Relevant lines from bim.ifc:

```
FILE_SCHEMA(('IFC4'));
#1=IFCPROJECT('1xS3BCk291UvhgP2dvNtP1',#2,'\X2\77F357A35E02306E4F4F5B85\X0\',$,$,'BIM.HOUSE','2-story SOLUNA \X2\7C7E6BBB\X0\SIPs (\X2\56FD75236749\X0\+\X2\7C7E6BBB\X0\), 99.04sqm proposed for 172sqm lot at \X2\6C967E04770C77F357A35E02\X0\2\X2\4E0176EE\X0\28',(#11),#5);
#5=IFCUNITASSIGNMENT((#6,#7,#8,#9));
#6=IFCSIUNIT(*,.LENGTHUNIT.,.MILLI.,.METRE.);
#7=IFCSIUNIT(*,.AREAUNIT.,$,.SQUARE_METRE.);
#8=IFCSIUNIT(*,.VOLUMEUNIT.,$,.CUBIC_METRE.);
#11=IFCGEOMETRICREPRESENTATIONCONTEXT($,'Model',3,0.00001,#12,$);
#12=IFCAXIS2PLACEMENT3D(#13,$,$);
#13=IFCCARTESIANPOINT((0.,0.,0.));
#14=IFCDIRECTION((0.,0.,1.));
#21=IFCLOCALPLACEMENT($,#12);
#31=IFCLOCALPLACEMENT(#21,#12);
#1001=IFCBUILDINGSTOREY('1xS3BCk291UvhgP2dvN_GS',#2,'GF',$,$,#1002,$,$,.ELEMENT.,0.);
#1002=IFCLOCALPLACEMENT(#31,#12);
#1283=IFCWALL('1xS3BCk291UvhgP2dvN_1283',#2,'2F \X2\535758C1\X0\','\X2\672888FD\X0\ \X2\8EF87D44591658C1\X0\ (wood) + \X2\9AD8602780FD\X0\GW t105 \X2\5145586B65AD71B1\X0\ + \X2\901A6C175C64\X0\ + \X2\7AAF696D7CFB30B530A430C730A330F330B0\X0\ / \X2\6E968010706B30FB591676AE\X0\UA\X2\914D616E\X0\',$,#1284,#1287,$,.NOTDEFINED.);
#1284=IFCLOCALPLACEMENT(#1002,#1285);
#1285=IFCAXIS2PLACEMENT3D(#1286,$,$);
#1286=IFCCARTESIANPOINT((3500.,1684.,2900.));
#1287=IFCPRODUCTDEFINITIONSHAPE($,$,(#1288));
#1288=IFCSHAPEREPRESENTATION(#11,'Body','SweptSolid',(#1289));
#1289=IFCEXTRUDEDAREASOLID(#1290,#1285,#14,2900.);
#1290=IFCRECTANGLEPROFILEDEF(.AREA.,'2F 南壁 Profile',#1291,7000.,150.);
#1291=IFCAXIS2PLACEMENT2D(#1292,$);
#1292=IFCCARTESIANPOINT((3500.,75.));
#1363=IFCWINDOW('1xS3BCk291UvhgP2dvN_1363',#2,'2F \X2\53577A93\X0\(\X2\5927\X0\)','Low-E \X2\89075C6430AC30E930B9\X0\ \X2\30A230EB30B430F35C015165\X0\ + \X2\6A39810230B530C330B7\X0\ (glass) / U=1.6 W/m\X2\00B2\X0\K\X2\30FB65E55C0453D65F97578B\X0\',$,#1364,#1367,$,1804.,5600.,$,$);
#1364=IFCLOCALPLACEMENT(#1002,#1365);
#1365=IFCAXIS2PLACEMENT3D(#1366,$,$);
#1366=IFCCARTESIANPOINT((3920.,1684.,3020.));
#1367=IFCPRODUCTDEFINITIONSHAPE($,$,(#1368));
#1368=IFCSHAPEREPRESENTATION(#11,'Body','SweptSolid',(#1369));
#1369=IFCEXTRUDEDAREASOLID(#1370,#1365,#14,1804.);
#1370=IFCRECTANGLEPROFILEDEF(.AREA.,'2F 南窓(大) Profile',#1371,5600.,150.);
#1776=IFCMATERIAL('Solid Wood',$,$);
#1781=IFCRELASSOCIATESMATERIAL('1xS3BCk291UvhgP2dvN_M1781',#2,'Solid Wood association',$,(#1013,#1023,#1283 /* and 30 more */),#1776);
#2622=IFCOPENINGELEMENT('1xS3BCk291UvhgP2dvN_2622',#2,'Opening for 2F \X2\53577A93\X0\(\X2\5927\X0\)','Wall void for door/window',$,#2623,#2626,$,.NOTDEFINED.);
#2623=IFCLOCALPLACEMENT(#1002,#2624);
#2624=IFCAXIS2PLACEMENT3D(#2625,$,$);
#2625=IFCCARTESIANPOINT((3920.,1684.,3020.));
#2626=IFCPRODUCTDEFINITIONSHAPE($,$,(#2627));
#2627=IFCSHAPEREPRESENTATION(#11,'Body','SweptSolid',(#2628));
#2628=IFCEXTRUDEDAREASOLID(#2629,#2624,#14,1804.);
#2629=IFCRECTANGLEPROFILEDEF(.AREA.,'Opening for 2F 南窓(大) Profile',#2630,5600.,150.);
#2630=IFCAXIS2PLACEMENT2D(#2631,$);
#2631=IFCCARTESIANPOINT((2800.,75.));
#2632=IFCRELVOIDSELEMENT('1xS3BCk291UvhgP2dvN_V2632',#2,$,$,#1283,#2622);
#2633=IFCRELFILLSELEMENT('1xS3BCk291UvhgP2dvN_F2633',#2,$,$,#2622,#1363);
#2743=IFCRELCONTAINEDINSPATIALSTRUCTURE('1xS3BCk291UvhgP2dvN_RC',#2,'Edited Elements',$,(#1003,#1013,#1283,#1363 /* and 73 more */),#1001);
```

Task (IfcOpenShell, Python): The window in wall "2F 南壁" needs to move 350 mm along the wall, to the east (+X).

```python
import ifcopenshell
import ifcopenshell.api.geometry
import ifcopenshell.util.placement
import ifcopenshell.util.unit

model = ifcopenshell.open("bim.ifc")
unit_scale = ifcopenshell.util.unit.calculate_unit_scale(model)

window = model.by_guid("1xS3BCk291UvhgP2dvN_1363")
opening = window.FillsVoids[0].RelatingOpeningElement
wall = opening.VoidsElements[0].RelatingBuildingElement

wall_matrix = ifcopenshell.util.placement.get_local_placement(wall.ObjectPlacement)
shift = wall_matrix[:3, 0] * 0.35 / unit_scale
before = ifcopenshell.util.placement.get_local_placement(window.ObjectPlacement)[:3, 3].copy()

# The window is not placed relative to its opening, so move both.
for product in (opening, window):
    matrix = ifcopenshell.util.placement.get_local_placement(product.ObjectPlacement)
    matrix[:3, 3] += shift
    ifcopenshell.api.geometry.edit_object_placement(model, product=product, matrix=matrix, is_si=False)

after = ifcopenshell.util.placement.get_local_placement(window.ObjectPlacement)[:3, 3]
print("window moved by", (after - before).round(3) + 0.0)

model.write("bim_updated.ifc")
```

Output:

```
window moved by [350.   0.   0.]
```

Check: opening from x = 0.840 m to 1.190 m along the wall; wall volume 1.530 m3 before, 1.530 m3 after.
